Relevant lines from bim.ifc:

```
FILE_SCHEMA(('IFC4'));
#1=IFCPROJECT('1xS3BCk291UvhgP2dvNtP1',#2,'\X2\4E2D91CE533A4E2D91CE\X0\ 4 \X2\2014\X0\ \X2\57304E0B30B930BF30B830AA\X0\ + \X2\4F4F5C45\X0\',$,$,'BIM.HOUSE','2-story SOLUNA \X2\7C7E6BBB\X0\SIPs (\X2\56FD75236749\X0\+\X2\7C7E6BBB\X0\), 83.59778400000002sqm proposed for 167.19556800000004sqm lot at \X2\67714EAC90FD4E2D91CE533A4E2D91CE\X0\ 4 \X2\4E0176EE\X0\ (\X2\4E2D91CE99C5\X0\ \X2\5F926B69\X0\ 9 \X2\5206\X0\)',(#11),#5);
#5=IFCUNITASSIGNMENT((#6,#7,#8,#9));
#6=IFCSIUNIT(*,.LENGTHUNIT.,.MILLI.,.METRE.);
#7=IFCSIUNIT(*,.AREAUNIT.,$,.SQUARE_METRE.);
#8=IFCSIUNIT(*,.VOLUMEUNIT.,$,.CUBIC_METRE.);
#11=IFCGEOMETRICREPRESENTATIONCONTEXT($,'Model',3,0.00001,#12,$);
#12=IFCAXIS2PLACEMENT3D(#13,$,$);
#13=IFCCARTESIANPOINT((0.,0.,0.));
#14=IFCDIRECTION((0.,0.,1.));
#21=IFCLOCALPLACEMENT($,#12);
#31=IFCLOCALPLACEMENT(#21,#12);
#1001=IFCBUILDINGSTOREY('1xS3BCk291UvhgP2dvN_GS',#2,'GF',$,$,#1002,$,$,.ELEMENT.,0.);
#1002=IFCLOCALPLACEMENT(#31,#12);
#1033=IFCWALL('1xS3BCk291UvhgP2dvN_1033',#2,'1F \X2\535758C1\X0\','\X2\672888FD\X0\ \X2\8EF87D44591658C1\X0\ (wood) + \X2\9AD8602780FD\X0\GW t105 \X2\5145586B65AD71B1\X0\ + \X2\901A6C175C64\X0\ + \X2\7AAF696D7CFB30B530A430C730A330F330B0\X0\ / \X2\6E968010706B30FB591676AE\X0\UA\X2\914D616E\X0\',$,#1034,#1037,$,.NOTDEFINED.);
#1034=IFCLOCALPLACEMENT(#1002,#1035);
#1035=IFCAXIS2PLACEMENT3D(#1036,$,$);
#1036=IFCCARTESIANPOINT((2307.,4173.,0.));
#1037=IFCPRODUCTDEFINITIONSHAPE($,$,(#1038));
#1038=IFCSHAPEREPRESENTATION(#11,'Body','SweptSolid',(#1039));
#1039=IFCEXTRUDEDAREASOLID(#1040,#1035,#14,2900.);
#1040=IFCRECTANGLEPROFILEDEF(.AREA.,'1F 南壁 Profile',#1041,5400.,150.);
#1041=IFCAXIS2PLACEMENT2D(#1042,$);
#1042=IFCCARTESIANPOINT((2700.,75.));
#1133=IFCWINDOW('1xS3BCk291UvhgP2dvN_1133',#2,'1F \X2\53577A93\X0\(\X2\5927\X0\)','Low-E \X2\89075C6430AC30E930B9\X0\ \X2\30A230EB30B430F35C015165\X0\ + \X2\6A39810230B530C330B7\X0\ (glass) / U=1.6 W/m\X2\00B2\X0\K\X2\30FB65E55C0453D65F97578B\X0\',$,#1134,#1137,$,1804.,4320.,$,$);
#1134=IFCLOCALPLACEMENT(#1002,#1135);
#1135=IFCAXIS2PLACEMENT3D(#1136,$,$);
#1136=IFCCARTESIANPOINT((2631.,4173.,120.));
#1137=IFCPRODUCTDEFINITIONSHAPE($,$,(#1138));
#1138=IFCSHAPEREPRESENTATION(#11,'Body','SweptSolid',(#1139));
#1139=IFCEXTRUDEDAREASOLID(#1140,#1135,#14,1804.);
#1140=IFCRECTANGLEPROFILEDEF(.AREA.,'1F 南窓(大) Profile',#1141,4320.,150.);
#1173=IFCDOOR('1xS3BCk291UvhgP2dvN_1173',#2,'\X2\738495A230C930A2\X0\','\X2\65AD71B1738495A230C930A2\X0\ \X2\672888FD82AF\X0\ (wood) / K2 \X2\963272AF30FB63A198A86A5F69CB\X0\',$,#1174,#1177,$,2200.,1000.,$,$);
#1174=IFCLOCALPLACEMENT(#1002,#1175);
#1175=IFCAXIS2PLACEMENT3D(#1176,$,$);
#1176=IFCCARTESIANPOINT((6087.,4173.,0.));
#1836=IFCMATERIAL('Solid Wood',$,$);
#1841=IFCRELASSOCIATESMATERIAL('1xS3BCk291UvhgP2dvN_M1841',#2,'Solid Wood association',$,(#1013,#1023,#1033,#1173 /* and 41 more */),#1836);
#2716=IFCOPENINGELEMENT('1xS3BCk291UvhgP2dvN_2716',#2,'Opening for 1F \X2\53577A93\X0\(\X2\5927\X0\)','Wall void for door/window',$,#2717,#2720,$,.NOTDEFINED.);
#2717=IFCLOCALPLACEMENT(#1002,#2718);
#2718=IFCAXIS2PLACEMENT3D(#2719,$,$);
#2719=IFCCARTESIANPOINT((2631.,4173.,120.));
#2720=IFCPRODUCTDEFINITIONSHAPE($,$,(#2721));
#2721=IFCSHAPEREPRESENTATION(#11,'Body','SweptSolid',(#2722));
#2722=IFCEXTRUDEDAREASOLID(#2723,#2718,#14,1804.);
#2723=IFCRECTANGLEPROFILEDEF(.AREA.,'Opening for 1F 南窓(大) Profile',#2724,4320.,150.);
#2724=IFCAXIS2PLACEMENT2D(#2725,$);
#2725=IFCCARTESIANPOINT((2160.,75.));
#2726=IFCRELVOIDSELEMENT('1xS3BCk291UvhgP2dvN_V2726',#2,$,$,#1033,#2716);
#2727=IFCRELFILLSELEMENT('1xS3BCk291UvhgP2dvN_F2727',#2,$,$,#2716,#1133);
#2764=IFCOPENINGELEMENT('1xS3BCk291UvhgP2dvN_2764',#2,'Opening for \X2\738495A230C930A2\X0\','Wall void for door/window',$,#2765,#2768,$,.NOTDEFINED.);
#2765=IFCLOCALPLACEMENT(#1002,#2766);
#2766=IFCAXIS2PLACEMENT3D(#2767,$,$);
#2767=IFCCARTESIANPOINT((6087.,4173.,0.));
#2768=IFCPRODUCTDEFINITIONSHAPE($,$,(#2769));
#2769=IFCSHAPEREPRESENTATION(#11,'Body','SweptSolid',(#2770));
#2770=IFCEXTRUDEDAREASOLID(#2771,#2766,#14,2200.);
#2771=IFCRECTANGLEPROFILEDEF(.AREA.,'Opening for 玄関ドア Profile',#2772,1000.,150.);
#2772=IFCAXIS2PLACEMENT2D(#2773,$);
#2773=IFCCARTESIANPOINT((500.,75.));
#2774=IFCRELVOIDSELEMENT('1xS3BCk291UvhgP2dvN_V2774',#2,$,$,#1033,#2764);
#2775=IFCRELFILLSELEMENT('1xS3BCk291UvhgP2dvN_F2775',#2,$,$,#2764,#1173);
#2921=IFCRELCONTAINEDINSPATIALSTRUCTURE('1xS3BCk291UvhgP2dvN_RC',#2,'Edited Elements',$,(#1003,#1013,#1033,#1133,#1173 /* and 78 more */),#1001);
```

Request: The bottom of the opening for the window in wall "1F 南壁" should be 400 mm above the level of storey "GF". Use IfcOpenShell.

```python
import numpy as np
import ifcopenshell
import ifcopenshell.api.geometry
import ifcopenshell.geom
import ifcopenshell.util.element
import ifcopenshell.util.placement
import ifcopenshell.util.shape
import ifcopenshell.util.unit

model = ifcopenshell.open("bim.ifc")
unit_scale = ifcopenshell.util.unit.calculate_unit_scale(model)

window = model.by_guid("1xS3BCk291UvhgP2dvN_1133")
opening = window.FillsVoids[0].RelatingOpeningElement
storey = ifcopenshell.util.element.get_container(window, ifc_class="IfcBuildingStorey")
level = ifcopenshell.util.placement.get_local_placement(storey.ObjectPlacement)[2, 3]

# The opening's origin need not be at the sill, so measure its lowest point.
shape = ifcopenshell.geom.create_shape(ifcopenshell.geom.settings(), opening)
bottom = ifcopenshell.util.shape.get_shape_bottom_elevation(shape, shape.geometry) / unit_scale
dz = level + 0.4 / unit_scale - bottom

shift = np.array([0.0, 0.0, dz])
# The window is not placed relative to its opening, so move both.
for product in (opening, window):
    matrix = ifcopenshell.util.placement.get_local_placement(product.ObjectPlacement)
    matrix[:3, 3] += shift
    ifcopenshell.api.geometry.edit_object_placement(model, product=product, matrix=matrix, is_si=False)

print(f"moved by {dz * unit_scale:+.3f} m")

model.write("bim_v2.ifc")
```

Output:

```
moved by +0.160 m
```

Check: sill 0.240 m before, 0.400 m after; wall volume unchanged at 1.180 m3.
